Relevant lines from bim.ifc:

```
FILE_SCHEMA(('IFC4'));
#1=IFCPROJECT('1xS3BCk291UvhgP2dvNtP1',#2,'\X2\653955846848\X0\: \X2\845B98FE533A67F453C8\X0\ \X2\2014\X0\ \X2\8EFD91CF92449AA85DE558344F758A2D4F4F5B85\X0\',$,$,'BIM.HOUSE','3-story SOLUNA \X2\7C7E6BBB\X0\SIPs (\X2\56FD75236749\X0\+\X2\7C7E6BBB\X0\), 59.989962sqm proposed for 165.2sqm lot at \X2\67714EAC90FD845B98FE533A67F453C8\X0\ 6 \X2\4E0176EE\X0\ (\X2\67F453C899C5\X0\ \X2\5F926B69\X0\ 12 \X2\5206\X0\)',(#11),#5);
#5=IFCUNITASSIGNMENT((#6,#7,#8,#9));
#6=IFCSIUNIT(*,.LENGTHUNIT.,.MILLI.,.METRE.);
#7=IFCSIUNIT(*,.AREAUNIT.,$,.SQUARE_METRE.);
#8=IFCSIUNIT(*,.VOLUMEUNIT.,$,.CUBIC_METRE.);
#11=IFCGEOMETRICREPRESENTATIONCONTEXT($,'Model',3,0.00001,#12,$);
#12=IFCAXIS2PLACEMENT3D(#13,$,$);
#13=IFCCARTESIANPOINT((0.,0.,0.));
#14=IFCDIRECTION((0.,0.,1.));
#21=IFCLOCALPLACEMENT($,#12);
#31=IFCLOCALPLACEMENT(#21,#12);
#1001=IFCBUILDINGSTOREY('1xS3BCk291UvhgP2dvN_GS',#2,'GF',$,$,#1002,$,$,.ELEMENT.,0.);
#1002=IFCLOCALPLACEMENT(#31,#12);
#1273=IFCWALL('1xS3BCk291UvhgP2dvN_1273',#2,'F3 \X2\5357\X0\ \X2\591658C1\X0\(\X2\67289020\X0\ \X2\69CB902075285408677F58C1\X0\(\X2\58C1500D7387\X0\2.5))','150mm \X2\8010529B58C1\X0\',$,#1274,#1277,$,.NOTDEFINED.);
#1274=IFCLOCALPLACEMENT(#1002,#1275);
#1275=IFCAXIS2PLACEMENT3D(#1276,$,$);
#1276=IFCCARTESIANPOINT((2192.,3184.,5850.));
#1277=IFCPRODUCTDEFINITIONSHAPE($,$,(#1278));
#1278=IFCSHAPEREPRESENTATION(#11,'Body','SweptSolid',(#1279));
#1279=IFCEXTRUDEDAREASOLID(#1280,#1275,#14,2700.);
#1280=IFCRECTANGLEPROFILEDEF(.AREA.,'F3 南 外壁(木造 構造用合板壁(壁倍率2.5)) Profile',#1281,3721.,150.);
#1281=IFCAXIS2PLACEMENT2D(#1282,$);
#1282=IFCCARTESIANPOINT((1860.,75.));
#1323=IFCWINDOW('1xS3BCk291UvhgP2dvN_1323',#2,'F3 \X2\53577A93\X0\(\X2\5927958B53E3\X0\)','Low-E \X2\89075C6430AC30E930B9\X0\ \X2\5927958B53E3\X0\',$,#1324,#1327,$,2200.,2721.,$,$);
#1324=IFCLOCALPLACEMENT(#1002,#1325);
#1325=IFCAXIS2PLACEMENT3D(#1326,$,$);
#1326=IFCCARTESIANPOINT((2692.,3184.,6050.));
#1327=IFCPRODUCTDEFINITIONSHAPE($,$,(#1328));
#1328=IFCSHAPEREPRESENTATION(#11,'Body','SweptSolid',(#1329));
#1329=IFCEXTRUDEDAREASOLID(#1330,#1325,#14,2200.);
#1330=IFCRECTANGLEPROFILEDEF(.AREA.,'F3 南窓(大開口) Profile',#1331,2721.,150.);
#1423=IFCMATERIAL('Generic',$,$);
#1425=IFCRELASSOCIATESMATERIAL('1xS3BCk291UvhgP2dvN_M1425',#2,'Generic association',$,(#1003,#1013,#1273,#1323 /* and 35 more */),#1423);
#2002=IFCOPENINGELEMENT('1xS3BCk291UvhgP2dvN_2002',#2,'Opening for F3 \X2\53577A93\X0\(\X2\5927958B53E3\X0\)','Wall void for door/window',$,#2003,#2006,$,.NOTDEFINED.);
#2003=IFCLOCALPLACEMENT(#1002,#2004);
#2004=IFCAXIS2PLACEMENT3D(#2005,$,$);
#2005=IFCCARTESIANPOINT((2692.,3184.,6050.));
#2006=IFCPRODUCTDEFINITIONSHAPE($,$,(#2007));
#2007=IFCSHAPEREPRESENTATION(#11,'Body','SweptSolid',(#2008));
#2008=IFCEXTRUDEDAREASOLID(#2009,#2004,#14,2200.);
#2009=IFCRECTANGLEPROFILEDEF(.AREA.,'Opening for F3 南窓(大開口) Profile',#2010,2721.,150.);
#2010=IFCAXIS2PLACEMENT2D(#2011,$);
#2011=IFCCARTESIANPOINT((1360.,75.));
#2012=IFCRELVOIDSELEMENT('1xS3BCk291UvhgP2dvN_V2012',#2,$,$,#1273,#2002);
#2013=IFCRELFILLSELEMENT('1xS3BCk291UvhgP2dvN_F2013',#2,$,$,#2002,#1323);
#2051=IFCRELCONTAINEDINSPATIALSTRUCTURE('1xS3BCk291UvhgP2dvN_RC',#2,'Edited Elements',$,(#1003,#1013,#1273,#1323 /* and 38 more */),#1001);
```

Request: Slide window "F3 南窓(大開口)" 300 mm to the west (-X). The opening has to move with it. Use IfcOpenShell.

```python
import ifcopenshell
import ifcopenshell.api.geometry
import ifcopenshell.util.placement
import ifcopenshell.util.unit

model = ifcopenshell.open("bim.ifc")
unit_scale = ifcopenshell.util.unit.calculate_unit_scale(model)

window = model.by_guid("1xS3BCk291UvhgP2dvN_1323")
opening = window.FillsVoids[0].RelatingOpeningElement
wall = opening.VoidsElements[0].RelatingBuildingElement

wall_matrix = ifcopenshell.util.placement.get_local_placement(wall.ObjectPlacement)
shift = wall_matrix[:3, 0] * -0.3 / unit_scale
before = ifcopenshell.util.placement.get_local_placement(window.ObjectPlacement)[:3, 3].copy()

# The window is not placed relative to its opening, so move both.
for product in (opening, window):
    matrix = ifcopenshell.util.placement.get_local_placement(product.ObjectPlacement)
    matrix[:3, 3] += shift
    ifcopenshell.api.geometry.edit_object_placement(model, product=product, matrix=matrix, is_si=False)

after = ifcopenshell.util.placement.get_local_placement(window.ObjectPlacement)[:3, 3]
print("window moved by", (after - before).round(3) + 0.0)

model.write("bim_updated.ifc")
```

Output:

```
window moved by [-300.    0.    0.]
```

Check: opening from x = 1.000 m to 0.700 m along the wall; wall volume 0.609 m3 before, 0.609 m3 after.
